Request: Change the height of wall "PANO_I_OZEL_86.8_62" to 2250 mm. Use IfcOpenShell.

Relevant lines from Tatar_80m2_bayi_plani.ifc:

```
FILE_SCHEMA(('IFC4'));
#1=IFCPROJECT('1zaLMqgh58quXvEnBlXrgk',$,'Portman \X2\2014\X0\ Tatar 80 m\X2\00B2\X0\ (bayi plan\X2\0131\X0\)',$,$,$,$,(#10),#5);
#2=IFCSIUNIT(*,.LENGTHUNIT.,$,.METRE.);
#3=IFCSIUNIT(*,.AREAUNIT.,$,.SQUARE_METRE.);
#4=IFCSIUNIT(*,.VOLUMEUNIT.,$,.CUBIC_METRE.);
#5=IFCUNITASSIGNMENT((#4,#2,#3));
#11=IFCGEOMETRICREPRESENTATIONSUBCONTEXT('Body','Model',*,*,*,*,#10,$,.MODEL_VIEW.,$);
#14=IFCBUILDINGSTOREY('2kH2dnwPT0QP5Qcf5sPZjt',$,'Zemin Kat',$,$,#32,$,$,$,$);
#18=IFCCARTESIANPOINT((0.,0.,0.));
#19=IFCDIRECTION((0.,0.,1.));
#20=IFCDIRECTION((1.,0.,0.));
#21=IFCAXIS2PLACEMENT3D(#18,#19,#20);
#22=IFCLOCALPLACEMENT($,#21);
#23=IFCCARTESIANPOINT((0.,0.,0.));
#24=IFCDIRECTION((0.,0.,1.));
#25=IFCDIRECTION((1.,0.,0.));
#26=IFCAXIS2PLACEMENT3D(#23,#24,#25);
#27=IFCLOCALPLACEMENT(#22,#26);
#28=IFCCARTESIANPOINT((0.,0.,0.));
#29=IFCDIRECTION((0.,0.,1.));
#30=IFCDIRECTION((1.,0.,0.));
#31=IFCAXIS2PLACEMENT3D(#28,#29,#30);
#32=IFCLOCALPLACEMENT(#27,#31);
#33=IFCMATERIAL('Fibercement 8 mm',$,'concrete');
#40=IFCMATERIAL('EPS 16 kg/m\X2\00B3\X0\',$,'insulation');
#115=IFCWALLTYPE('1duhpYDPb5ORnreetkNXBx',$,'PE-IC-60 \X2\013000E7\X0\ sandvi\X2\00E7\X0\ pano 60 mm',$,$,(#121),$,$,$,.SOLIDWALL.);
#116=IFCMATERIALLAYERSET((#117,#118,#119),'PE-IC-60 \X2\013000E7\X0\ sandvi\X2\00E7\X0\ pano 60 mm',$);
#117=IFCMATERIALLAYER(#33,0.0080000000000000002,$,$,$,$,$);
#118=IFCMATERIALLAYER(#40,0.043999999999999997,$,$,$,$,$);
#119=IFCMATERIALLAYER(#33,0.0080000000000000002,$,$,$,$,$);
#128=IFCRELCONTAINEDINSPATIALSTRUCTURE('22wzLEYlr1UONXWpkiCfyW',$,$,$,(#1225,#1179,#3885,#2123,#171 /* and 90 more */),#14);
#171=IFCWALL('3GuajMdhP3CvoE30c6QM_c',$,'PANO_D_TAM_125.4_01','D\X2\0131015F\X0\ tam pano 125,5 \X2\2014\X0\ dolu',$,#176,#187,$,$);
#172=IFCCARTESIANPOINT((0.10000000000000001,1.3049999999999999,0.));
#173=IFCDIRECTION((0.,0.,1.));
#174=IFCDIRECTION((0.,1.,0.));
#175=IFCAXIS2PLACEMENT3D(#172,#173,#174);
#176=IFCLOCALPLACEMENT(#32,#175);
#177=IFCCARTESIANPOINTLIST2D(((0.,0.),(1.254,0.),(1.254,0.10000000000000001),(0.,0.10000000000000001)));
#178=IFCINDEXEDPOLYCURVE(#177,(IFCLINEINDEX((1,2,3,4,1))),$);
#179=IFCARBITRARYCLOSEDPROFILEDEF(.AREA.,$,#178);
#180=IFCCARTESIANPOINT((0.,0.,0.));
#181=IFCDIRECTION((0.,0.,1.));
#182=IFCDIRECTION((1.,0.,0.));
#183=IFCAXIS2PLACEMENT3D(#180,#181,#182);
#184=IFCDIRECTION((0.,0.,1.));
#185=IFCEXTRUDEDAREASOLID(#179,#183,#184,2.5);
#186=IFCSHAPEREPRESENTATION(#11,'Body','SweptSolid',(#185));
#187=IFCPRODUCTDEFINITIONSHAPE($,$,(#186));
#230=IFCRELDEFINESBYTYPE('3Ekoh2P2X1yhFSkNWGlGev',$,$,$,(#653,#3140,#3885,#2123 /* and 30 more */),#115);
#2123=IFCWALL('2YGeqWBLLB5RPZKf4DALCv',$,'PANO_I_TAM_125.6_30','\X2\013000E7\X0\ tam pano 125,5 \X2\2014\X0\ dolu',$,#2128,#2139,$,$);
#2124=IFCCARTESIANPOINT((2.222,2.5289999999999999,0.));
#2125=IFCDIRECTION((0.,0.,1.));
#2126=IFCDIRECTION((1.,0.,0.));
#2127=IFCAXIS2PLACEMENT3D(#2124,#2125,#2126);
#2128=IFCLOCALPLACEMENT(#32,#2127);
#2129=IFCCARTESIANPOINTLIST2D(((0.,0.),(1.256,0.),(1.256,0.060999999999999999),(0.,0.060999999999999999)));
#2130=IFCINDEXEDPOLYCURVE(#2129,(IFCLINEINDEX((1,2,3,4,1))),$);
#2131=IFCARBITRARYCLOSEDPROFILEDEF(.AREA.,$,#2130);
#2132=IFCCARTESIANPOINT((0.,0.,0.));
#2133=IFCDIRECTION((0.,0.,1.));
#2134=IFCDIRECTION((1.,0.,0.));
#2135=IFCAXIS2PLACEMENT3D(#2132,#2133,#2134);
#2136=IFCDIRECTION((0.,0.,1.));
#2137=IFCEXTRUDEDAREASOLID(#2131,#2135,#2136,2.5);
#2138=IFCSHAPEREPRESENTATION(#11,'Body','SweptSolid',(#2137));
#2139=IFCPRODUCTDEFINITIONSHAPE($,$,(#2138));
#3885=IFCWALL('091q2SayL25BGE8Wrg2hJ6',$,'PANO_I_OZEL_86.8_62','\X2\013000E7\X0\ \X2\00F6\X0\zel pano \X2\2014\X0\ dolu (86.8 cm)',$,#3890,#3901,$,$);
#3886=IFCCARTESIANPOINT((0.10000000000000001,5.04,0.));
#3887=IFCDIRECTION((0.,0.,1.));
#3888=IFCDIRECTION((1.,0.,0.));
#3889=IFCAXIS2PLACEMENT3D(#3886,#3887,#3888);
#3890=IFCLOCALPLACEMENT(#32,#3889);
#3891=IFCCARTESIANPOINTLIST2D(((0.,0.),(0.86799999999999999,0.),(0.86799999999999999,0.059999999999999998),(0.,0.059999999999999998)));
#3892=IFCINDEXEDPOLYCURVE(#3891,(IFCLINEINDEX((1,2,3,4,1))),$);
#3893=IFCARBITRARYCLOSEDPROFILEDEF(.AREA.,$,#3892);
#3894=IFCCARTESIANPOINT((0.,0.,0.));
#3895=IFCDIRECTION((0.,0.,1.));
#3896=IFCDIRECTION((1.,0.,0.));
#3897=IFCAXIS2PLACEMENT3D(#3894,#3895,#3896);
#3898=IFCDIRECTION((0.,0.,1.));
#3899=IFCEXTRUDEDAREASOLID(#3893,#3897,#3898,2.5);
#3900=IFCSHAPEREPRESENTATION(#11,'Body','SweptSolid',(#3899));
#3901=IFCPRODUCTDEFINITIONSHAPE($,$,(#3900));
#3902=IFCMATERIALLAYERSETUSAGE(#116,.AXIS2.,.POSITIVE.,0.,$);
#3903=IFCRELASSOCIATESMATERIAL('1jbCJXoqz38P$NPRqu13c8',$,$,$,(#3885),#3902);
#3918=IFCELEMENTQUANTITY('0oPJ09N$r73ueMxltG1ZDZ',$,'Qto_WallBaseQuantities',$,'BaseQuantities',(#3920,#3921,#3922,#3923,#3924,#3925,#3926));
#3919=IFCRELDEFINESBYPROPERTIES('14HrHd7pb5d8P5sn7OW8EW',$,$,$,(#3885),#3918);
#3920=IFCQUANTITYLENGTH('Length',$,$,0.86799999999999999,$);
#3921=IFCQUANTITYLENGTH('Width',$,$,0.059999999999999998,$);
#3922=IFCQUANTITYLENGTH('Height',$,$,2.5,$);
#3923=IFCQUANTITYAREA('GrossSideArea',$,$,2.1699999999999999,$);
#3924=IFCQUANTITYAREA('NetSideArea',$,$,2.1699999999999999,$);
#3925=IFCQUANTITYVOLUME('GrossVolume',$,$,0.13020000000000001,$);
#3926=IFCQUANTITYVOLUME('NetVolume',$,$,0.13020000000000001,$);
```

```python
import ifcopenshell
import ifcopenshell.api.pset
import ifcopenshell.geom
import ifcopenshell.util.element
import ifcopenshell.util.representation
import ifcopenshell.util.shape
import ifcopenshell.util.unit

model = ifcopenshell.open("Tatar_80m2_bayi_plani.ifc")
unit_scale = ifcopenshell.util.unit.calculate_unit_scale(model)
area_scale = ifcopenshell.util.unit.calculate_unit_scale(model, "AREAUNIT")
volume_scale = ifcopenshell.util.unit.calculate_unit_scale(model, "VOLUMEUNIT")
settings = ifcopenshell.geom.settings()


def volume(element):
    """Net volume in cubic metres, openings subtracted."""
    shape = ifcopenshell.geom.create_shape(settings, element)
    return ifcopenshell.util.shape.get_volume(shape.geometry)


wall = model.by_guid("091q2SayL25BGE8Wrg2hJ6")
before = volume(wall)

body = ifcopenshell.util.representation.get_representation(wall, "Model", "Body")
solid = body.Items[0]
old_height = solid.Depth
solid.Depth = 2.25 / unit_scale
after = volume(wall)
thickness = 0.06  # wall thickness in metres

# Update the stored height, areas and volumes.
qto = model.by_id(ifcopenshell.util.element.get_pset(wall, "Qto_WallBaseQuantities", should_inherit=False)["id"])
ifcopenshell.api.pset.edit_qto(model, qto=qto, properties={
    "Height": solid.Depth,
    "GrossSideArea": ifcopenshell.util.element.get_pset(wall, "Qto_WallBaseQuantities", "GrossSideArea") * solid.Depth / old_height,
    "NetSideArea": after / thickness / area_scale,
    "GrossVolume": ifcopenshell.util.element.get_pset(wall, "Qto_WallBaseQuantities", "GrossVolume") * solid.Depth / old_height,
    "NetVolume": after / volume_scale,
})

print(f"height {old_height:g} -> {solid.Depth:g}, volume {before:.3f} -> {after:.3f} m3")

model.write("Tatar_80m2_bayi_plani_edited.ifc")
```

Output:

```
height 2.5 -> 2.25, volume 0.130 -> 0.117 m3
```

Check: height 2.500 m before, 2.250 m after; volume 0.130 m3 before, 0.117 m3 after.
